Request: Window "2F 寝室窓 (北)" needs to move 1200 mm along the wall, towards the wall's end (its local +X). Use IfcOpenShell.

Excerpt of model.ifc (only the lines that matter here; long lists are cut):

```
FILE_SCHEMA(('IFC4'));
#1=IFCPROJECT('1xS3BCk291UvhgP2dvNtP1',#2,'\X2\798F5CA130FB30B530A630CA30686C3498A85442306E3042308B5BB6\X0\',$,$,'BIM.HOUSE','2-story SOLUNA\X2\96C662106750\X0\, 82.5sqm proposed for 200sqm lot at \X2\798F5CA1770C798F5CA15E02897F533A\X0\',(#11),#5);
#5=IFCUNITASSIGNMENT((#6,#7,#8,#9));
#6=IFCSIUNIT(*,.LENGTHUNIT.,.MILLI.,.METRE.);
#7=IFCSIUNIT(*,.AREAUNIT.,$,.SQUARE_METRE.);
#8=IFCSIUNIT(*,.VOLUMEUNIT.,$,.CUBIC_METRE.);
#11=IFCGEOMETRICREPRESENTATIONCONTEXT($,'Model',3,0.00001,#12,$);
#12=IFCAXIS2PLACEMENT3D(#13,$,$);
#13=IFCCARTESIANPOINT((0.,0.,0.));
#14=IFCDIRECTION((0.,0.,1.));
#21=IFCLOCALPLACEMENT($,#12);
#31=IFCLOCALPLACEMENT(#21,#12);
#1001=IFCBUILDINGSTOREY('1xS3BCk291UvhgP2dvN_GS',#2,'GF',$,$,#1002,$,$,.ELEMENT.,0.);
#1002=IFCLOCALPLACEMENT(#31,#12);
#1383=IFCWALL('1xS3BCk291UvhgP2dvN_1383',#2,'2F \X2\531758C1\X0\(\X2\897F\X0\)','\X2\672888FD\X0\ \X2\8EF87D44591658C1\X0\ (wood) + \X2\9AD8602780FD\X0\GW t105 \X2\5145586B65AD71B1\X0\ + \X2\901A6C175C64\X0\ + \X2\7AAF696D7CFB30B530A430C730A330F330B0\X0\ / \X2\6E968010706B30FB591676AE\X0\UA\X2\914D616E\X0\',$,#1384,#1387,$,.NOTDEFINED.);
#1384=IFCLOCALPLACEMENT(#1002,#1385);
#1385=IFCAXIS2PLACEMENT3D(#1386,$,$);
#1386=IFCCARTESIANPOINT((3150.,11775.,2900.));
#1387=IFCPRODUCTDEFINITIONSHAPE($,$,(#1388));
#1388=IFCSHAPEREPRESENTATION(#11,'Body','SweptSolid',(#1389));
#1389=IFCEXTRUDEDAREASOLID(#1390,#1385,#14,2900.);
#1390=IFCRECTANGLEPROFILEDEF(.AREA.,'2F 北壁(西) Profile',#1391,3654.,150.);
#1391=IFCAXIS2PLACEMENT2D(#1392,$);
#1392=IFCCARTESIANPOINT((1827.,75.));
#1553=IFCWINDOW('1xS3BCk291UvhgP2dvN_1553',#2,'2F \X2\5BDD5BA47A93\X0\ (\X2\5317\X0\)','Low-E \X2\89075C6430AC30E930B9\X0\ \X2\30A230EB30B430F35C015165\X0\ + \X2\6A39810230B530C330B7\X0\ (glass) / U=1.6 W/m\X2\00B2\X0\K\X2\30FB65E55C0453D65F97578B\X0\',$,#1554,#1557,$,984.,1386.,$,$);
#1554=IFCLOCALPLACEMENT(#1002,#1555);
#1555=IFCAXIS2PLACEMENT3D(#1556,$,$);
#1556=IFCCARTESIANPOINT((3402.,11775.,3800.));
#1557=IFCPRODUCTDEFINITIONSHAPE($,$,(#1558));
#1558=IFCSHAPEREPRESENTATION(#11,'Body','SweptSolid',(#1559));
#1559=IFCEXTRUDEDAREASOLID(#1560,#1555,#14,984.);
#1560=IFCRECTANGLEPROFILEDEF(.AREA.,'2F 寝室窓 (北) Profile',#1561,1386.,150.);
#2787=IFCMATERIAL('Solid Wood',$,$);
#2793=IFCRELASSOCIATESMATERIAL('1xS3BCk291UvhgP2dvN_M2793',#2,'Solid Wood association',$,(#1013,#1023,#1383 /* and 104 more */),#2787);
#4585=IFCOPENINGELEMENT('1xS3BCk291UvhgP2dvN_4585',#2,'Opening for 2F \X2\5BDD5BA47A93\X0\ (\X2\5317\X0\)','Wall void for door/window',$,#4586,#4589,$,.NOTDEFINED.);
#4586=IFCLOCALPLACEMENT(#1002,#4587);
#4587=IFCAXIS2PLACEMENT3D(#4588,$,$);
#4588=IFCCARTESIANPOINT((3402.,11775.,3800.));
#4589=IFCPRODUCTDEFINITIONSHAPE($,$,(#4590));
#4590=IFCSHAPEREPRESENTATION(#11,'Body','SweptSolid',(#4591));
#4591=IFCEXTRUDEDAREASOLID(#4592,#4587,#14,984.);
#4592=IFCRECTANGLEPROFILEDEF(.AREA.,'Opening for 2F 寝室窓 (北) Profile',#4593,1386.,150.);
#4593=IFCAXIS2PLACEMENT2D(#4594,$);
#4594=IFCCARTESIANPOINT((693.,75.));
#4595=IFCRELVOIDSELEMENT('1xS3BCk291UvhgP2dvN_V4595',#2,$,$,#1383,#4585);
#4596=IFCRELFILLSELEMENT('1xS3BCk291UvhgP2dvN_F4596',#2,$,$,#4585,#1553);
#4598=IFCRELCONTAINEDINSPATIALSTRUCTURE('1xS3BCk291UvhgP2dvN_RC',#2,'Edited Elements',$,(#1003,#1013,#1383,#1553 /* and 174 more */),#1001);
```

```python
import ifcopenshell
import ifcopenshell.api.geometry
import ifcopenshell.util.placement
import ifcopenshell.util.unit

model = ifcopenshell.open("model.ifc")
unit_scale = ifcopenshell.util.unit.calculate_unit_scale(model)

window = model.by_guid("1xS3BCk291UvhgP2dvN_1553")
opening = window.FillsVoids[0].RelatingOpeningElement
wall = opening.VoidsElements[0].RelatingBuildingElement

wall_matrix = ifcopenshell.util.placement.get_local_placement(wall.ObjectPlacement)
shift = wall_matrix[:3, 0] * 1.2 / unit_scale
before = ifcopenshell.util.placement.get_local_placement(window.ObjectPlacement)[:3, 3].copy()

# The window is not placed relative to its opening, so move both.
for product in (opening, window):
    matrix = ifcopenshell.util.placement.get_local_placement(product.ObjectPlacement)
    matrix[:3, 3] += shift
    ifcopenshell.api.geometry.edit_object_placement(model, product=product, matrix=matrix, is_si=False)

after = ifcopenshell.util.placement.get_local_placement(window.ObjectPlacement)[:3, 3]
print("window moved by", (after - before).round(3) + 0.0)

model.write("model_updated.ifc")
```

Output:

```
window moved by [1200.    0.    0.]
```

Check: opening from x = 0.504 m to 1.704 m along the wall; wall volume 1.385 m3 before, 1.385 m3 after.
